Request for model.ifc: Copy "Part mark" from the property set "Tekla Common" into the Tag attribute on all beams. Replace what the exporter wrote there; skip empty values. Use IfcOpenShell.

First a look at what the model holds.

```python
import ifcopenshell
import ifcopenshell.util.element

model = ifcopenshell.open("model.ifc")
print(model.schema)
beams = model.by_type("IfcBeam")
print(len(beams), "beams")
for e in beams[:8]:
    source = ifcopenshell.util.element.get_pset(e, "Tekla Common", "Part mark")
    target = e.Tag
    print(e.id(), repr(source), repr(target), sep=" | ")
```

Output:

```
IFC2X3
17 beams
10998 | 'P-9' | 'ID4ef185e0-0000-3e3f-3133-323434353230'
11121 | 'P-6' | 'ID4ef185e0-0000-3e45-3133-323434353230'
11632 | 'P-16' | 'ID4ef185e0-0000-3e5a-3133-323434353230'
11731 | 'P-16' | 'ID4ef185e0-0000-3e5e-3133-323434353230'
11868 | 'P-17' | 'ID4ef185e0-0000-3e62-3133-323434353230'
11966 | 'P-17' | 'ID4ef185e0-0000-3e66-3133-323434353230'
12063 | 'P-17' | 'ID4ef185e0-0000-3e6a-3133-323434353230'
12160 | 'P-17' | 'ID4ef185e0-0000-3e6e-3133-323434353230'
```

```python
import ifcopenshell
import ifcopenshell.util.element

model = ifcopenshell.open("model.ifc")

count = 0
for e in model.by_type("IfcBeam"):
    value = ifcopenshell.util.element.get_pset(e, "Tekla Common", "Part mark")
    current = e.Tag
    if not value or not value.strip() or current == value:
        continue
    e.Tag = value
    count += 1

print(count, "beams updated")

model.write("model_edited.ifc")
```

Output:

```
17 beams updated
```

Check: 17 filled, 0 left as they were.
